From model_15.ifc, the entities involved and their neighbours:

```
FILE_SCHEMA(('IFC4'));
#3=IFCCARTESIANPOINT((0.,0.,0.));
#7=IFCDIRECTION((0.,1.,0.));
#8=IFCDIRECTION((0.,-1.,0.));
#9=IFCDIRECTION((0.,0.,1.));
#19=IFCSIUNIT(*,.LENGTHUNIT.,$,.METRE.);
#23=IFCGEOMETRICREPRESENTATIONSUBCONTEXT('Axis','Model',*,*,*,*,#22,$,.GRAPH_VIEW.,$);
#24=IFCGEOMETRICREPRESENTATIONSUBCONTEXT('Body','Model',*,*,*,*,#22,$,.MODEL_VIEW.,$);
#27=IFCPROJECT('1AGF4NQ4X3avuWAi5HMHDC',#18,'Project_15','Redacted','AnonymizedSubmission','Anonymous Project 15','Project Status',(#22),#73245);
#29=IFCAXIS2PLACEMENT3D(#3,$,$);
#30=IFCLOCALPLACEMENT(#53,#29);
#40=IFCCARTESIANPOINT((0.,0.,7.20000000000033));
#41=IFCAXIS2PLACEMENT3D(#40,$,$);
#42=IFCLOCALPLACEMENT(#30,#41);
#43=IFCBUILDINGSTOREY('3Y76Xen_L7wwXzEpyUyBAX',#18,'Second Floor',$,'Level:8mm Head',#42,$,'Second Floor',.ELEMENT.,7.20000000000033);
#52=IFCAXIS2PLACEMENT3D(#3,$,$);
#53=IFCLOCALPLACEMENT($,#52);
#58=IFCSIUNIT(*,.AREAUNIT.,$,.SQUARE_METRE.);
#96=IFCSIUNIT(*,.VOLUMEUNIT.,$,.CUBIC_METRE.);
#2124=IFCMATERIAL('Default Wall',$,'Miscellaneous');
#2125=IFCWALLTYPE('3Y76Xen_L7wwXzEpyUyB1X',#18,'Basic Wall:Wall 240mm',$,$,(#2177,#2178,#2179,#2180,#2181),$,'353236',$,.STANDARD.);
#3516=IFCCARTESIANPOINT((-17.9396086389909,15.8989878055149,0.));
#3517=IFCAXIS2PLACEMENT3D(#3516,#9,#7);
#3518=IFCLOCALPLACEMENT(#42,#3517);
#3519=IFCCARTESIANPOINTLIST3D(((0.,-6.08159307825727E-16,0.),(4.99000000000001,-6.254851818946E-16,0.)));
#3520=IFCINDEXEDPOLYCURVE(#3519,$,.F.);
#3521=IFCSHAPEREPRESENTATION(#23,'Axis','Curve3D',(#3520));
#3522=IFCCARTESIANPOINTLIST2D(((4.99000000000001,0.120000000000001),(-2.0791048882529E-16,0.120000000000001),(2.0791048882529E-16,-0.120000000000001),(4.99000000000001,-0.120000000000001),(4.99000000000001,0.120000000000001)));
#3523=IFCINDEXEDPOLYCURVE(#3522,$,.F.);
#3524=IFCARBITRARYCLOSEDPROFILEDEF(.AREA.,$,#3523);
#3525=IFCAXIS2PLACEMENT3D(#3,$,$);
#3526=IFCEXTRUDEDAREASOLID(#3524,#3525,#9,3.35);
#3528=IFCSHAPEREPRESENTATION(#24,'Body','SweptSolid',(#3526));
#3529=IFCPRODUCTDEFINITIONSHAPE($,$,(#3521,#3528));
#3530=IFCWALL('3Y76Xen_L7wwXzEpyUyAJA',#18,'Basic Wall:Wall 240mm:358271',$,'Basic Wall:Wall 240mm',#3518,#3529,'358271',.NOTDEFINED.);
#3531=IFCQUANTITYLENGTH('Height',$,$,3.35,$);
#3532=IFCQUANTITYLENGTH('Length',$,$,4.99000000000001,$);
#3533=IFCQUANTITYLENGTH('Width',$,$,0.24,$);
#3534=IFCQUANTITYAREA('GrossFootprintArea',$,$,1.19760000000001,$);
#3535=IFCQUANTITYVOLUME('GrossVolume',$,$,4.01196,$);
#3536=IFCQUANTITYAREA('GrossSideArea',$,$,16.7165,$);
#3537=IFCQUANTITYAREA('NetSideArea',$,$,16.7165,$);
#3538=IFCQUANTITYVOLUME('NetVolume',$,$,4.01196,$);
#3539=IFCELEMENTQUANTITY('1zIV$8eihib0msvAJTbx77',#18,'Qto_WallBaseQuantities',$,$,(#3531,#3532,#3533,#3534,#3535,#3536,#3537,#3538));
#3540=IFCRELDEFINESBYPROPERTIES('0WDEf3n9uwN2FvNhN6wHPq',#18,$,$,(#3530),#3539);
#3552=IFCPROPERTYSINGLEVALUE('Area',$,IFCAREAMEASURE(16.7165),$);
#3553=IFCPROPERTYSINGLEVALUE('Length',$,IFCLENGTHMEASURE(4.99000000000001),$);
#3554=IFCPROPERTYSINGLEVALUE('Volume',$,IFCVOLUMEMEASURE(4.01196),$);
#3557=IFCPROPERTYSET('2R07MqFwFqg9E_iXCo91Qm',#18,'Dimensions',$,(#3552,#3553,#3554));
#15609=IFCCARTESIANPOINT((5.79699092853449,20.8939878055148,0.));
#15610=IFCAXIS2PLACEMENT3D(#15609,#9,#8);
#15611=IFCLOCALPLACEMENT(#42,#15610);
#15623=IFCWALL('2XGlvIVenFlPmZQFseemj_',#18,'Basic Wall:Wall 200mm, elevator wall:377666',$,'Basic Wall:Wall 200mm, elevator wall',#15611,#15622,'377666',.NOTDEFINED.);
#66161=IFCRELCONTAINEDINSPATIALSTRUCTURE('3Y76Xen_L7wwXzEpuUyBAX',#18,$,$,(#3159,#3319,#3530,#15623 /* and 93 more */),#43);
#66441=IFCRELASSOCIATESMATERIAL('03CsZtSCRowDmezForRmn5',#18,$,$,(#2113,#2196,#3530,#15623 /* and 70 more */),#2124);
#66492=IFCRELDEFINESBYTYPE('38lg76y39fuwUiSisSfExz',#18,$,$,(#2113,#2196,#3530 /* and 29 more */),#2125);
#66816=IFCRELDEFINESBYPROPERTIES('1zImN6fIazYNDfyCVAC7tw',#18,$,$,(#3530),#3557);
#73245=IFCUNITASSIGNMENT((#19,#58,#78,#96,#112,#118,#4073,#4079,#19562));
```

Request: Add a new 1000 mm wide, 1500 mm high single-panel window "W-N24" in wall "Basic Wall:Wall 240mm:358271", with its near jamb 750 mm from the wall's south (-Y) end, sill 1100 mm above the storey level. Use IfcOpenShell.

```python
import numpy as np
import ifcopenshell
import ifcopenshell.api.feature
import ifcopenshell.api.geometry
import ifcopenshell.api.pset
import ifcopenshell.api.root
import ifcopenshell.api.spatial
import ifcopenshell.geom
import ifcopenshell.util.element
import ifcopenshell.util.placement
import ifcopenshell.util.representation
import ifcopenshell.util.shape
import ifcopenshell.util.unit

model = ifcopenshell.open("model_15.ifc")
unit_scale = ifcopenshell.util.unit.calculate_unit_scale(model)
area_scale = ifcopenshell.util.unit.calculate_unit_scale(model, "AREAUNIT")
volume_scale = ifcopenshell.util.unit.calculate_unit_scale(model, "VOLUMEUNIT")
settings = ifcopenshell.geom.settings()


def volume(element):
    """Net volume in cubic metres, openings subtracted."""
    shape = ifcopenshell.geom.create_shape(settings, element)
    return ifcopenshell.util.shape.get_volume(shape.geometry)


wall = model.by_guid("3Y76Xen_L7wwXzEpyUyAJA")
storey = ifcopenshell.util.element.get_container(wall, ifc_class="IfcBuildingStorey")
context = ifcopenshell.util.representation.get_context(model, "Model", "Body", "MODEL_VIEW")
before = volume(wall)

width, height, from_end, sill = 1, 1.5, 0.75, 1.1  # metres

# The wall runs along its own X axis, and the end named is its -X end.
wall_shape = ifcopenshell.geom.create_shape(settings, wall)
x, y, z = ifcopenshell.util.shape.get_vertices(wall_shape.geometry).T
start = x.min() + from_end
face, thickness = float(y.min()), float(y.max() - y.min())
wall_matrix = ifcopenshell.util.placement.get_local_placement(wall.ObjectPlacement)
level = ifcopenshell.util.placement.get_local_placement(storey.ObjectPlacement)[2, 3]


def in_wall(x, y):
    """Placement at x, y metres in the wall's axes, at sill height."""
    matrix = wall_matrix.copy()
    matrix[:, 3] = wall_matrix @ np.array([x / unit_scale, y / unit_scale, 0.0, 1.0])
    matrix[2, 3] = level + sill / unit_scale
    return matrix


# Opening: a box that overshoots both wall faces by 50 mm.
opening = ifcopenshell.api.root.create_entity(model, ifc_class="IfcOpeningElement", predefined_type="OPENING")
box = ifcopenshell.api.geometry.add_wall_representation(
    model, context=context, length=width, height=height, thickness=thickness + 0.1
)
ifcopenshell.api.geometry.assign_representation(model, product=opening, representation=box)
ifcopenshell.api.geometry.edit_object_placement(model, product=opening, matrix=in_wall(start, face - 0.05), is_si=False)
ifcopenshell.api.feature.add_feature(model, feature=opening, element=wall)

window = ifcopenshell.api.root.create_entity(model, ifc_class="IfcWindow", name="W-N24", predefined_type="WINDOW")
window.OverallWidth, window.OverallHeight = width / unit_scale, height / unit_scale
window.PartitioningType = "SINGLE_PANEL"
body = ifcopenshell.api.geometry.add_window_representation(
    model,
    context=context,
    overall_width=window.OverallWidth,
    overall_height=window.OverallHeight,
    partition_type="SINGLE_PANEL",
)
ifcopenshell.api.geometry.assign_representation(model, product=window, representation=body)
ifcopenshell.api.spatial.assign_container(model, products=[window], relating_structure=storey)
ifcopenshell.api.feature.add_filling(model, opening=opening, element=window)

# Centre the window in the wall's thickness.
ifcopenshell.api.geometry.edit_object_placement(model, product=window, matrix=in_wall(start, face), is_si=False)
window_shape = ifcopenshell.geom.create_shape(settings, window)
depth = ifcopenshell.util.shape.get_vertices(window_shape.geometry)[:, 1]
offset = face + thickness / 2 - (depth.min() + depth.max()) / 2
ifcopenshell.api.geometry.edit_object_placement(model, product=window, matrix=in_wall(start, offset), is_si=False)

after = volume(wall)

# Update the wall's stored quantities.
qto = model.by_id(ifcopenshell.util.element.get_pset(wall, "Qto_WallBaseQuantities", should_inherit=False)["id"])
ifcopenshell.api.pset.edit_qto(model, qto=qto, properties={
    "NetSideArea": after / thickness / area_scale,
    "NetVolume": after / volume_scale,
})
pset = model.by_id(ifcopenshell.util.element.get_pset(wall, "Dimensions", should_inherit=False)["id"])
ifcopenshell.api.pset.edit_pset(model, pset=pset, properties={
    "Area": model.create_entity("IfcAreaMeasure", after / thickness / area_scale),
    "Volume": model.create_entity("IfcVolumeMeasure", after / volume_scale),
})

print(f"wall volume {before:.3f} -> {after:.3f} m3")

model.write("model_15_rev.ifc")
```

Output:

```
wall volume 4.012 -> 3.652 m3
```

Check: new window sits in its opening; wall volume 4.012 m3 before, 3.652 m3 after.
